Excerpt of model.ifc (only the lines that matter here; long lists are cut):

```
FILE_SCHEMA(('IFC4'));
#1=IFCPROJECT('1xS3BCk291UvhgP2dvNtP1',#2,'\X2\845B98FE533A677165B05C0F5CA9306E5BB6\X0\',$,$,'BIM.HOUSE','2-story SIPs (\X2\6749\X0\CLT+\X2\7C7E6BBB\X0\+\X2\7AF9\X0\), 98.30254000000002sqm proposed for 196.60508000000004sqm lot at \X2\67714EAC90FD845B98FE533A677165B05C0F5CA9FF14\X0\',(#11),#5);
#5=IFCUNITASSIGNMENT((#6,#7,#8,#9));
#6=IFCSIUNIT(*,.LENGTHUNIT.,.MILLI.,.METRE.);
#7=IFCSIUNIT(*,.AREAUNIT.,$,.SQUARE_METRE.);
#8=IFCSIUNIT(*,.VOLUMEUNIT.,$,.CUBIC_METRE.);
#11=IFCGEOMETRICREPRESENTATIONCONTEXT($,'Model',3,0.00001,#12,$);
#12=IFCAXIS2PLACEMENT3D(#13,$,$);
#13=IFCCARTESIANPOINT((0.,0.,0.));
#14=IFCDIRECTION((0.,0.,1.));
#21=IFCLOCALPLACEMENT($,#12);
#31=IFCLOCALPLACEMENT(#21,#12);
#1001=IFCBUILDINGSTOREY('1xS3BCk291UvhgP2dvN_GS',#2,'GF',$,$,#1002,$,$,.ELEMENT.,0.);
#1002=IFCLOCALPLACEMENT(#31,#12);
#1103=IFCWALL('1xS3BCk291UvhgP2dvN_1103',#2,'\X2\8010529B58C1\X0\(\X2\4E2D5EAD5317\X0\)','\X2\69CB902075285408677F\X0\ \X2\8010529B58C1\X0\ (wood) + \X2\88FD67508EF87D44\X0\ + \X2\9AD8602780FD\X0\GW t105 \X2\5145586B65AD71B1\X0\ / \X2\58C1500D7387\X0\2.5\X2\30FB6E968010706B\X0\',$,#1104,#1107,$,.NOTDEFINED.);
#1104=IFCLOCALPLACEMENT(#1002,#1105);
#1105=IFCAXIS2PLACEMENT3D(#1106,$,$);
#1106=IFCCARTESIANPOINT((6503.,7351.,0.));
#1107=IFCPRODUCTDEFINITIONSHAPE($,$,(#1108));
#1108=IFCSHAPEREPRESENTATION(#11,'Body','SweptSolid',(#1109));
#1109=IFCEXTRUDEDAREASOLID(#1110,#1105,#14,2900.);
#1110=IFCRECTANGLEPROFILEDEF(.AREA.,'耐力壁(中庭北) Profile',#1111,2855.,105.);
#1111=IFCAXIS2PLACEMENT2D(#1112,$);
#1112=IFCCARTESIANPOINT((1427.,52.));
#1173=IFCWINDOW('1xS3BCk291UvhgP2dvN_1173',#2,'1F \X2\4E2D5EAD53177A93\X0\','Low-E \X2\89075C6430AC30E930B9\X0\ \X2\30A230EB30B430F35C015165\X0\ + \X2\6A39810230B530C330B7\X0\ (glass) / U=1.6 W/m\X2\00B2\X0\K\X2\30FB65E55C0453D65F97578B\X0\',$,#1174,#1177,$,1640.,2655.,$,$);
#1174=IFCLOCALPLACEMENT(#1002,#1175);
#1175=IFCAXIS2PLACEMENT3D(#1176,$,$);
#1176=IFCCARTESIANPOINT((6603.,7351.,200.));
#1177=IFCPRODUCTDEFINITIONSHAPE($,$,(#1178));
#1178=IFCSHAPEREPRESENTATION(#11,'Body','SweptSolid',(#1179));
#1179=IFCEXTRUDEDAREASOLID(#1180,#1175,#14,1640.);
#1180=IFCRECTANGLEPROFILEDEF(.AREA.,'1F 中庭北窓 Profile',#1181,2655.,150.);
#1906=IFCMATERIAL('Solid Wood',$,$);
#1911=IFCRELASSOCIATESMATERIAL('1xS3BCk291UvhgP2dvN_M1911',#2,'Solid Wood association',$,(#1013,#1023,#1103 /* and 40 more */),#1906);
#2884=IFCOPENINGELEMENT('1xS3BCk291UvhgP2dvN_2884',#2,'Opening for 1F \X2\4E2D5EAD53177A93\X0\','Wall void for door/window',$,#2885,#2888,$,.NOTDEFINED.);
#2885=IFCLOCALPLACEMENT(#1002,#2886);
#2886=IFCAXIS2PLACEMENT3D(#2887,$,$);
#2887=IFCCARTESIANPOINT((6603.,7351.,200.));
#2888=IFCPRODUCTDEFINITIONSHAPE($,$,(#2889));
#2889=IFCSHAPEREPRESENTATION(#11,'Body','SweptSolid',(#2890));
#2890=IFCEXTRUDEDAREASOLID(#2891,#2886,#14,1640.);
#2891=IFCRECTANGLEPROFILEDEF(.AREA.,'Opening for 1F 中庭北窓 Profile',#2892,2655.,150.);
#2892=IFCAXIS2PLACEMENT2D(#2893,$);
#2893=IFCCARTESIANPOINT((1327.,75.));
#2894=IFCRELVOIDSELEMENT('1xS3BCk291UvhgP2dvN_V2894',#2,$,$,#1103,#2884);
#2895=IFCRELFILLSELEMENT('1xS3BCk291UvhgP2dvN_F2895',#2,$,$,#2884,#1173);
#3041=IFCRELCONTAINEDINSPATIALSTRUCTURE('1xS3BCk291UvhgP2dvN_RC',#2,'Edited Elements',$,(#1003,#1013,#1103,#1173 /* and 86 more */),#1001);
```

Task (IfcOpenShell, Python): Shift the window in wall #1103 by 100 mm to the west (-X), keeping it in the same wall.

```python
import ifcopenshell
import ifcopenshell.api.geometry
import ifcopenshell.util.placement

model = ifcopenshell.open("model.ifc")

window = model.by_id(1173)
opening = window.FillsVoids[0].RelatingOpeningElement
wall = opening.VoidsElements[0].RelatingBuildingElement

wall_matrix = ifcopenshell.util.placement.get_local_placement(wall.ObjectPlacement)
shift = wall_matrix[:3, 0] * -100.0
before = ifcopenshell.util.placement.get_local_placement(window.ObjectPlacement)[:3, 3].copy()

# The window is not placed relative to its opening, so move both.
for product in (opening, window):
    matrix = ifcopenshell.util.placement.get_local_placement(product.ObjectPlacement)
    matrix[:3, 3] += shift
    ifcopenshell.api.geometry.edit_object_placement(model, product=product, matrix=matrix, is_si=False)

after = ifcopenshell.util.placement.get_local_placement(window.ObjectPlacement)[:3, 3]
print("window moved by", (after - before).round(3) + 0.0)

model.write("model_edited.ifc")
```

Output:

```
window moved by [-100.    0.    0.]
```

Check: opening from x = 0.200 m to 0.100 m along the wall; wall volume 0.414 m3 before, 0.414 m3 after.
